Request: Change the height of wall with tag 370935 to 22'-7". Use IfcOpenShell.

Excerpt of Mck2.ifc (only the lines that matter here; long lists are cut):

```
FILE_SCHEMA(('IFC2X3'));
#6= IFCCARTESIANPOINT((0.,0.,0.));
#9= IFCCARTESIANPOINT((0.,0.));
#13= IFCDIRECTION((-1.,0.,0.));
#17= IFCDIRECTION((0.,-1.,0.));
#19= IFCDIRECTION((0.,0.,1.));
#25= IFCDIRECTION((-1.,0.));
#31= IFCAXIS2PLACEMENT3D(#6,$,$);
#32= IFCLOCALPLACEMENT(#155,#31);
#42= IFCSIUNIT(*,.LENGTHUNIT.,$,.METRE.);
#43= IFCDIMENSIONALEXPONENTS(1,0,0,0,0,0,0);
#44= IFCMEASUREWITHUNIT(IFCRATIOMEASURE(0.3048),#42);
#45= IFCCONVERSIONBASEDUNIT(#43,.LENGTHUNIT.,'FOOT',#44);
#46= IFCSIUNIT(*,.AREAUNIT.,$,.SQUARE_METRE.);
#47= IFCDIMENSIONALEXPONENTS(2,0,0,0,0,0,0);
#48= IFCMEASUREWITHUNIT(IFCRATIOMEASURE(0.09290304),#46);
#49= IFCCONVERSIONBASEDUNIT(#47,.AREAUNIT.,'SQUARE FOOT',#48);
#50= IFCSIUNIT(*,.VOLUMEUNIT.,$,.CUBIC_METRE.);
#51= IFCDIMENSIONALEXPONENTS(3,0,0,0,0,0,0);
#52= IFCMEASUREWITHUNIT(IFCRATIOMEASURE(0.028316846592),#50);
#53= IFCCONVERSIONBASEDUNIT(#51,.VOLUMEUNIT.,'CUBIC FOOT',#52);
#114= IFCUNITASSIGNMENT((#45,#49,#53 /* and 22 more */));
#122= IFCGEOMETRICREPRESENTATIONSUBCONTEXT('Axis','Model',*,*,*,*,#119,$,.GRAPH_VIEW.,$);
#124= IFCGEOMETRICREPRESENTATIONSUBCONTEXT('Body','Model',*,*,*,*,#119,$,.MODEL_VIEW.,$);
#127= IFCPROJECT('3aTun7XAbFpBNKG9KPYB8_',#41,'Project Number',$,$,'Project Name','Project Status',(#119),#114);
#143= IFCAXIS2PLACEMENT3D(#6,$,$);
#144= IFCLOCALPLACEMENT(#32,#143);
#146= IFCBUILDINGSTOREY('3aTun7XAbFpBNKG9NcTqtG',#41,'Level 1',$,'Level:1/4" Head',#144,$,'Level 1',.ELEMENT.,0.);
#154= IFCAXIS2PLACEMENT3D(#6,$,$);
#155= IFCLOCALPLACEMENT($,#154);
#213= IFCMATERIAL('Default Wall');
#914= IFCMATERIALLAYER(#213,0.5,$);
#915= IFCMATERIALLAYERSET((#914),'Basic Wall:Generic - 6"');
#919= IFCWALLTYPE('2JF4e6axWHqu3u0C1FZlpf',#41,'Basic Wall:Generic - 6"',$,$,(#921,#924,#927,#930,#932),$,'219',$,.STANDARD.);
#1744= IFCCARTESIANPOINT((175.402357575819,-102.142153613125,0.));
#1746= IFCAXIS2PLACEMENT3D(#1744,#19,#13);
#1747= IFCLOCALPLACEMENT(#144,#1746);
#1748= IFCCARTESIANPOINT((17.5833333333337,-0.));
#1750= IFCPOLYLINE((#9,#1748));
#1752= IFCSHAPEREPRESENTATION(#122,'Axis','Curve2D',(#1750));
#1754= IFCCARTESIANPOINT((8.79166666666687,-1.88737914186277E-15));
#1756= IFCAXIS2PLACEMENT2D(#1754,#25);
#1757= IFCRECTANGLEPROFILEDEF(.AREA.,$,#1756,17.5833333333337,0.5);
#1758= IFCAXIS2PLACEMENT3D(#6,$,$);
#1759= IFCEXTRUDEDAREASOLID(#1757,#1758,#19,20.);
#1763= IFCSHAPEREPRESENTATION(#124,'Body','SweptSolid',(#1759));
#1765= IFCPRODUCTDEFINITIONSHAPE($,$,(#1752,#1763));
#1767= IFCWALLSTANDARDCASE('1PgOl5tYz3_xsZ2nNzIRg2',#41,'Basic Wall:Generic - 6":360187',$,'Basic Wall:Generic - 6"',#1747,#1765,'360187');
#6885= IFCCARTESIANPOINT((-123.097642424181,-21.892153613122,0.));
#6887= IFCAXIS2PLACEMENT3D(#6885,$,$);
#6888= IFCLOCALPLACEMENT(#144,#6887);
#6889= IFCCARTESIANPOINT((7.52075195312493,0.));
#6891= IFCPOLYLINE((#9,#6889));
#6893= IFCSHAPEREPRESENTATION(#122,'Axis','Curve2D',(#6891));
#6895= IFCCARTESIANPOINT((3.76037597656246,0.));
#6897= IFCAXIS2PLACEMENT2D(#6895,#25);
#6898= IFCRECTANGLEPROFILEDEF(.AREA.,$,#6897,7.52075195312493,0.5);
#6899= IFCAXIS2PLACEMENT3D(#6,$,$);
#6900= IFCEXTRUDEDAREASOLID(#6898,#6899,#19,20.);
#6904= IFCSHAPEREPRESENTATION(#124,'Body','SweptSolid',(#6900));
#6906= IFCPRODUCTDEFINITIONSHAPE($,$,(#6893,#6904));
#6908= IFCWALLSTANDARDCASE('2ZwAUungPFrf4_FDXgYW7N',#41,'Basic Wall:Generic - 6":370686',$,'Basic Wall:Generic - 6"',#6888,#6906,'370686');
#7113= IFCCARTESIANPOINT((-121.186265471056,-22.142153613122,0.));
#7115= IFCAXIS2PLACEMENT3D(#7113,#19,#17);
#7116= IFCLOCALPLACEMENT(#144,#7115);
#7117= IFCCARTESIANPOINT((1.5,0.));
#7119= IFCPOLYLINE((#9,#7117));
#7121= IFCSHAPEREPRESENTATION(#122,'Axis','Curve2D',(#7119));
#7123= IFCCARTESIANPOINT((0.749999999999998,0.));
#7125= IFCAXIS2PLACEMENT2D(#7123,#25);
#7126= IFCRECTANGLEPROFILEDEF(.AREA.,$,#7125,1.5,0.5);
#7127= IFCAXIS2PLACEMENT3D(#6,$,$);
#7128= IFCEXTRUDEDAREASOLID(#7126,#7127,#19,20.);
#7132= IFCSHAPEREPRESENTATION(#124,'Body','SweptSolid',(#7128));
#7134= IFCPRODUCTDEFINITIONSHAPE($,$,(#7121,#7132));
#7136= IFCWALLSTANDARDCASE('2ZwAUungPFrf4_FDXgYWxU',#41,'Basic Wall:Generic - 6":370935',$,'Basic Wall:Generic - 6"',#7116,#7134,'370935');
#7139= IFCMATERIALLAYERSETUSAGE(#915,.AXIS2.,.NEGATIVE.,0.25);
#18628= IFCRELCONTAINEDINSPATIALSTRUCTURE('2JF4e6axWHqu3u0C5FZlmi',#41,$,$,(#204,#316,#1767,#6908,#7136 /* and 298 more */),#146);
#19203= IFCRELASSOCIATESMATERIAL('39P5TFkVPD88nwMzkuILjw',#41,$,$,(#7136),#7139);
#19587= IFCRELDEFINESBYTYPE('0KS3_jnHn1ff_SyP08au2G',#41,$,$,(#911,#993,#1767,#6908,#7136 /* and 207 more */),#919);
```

```python
import ifcopenshell
import ifcopenshell.geom
import ifcopenshell.util.representation
import ifcopenshell.util.shape
import ifcopenshell.util.unit

model = ifcopenshell.open("Mck2.ifc")
unit_scale = ifcopenshell.util.unit.calculate_unit_scale(model)
settings = ifcopenshell.geom.settings()


def volume(element):
    """Net volume in cubic metres, openings subtracted."""
    shape = ifcopenshell.geom.create_shape(settings, element)
    return ifcopenshell.util.shape.get_volume(shape.geometry)


wall = model.by_guid("2ZwAUungPFrf4_FDXgYWxU")
before = volume(wall)

body = ifcopenshell.util.representation.get_representation(wall, "Model", "Body")
solid = body.Items[0]
old_height = solid.Depth
solid.Depth = 271 * 0.0254 / unit_scale
after = volume(wall)

print(f"height {old_height:g} -> {solid.Depth:g}, volume {before:.3f} -> {after:.3f} m3")

model.write("Mck2_updated.ifc")
```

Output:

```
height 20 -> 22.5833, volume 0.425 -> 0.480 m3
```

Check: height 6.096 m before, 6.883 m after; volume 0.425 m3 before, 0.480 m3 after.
